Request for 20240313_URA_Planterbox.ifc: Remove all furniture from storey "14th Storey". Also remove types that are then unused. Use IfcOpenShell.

First a look at what the model holds.

```python
import ifcopenshell
import ifcopenshell.util.element

model = ifcopenshell.open("20240313_URA_Planterbox.ifc")
print(model.schema)
storey = next(s for s in model.by_type("IfcBuildingStorey") if s.Name == "14th Storey")
furniture = [e for e in ifcopenshell.util.element.get_decomposition(storey) if e.is_a("IfcFurnishingElement")]
seen = {}
for e in furniture:
    element_type = ifcopenshell.util.element.get_type(e)
    name = element_type.Name if element_type not in (None, e) else None
    seen[name] = seen.get(name, 0) + 1
for name, count in sorted(seen.items(), key=str):
    print(count, "x", name)
```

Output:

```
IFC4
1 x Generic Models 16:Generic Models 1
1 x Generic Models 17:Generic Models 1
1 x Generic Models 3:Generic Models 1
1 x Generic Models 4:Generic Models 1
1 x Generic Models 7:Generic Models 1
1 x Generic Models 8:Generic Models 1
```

```python
import ifcopenshell
import ifcopenshell.api.root
import ifcopenshell.util.element

model = ifcopenshell.open("20240313_URA_Planterbox.ifc")

storey = next(s for s in model.by_type("IfcBuildingStorey") if s.Name == "14th Storey")
furniture = [e for e in ifcopenshell.util.element.get_decomposition(storey) if e.is_a("IfcFurnishingElement")]
types = {ifcopenshell.util.element.get_type(e) for e in furniture} - {None, *furniture}

for e in furniture:
    ifcopenshell.api.root.remove_product(model, product=e)
print(len(furniture), "removed")

unused = [t for t in types if not ifcopenshell.util.element.get_types(t)]
for t in unused:
    ifcopenshell.api.root.remove_product(model, product=t)
print(len(unused), "unused types removed")

model.write("20240313_URA_Planterbox_rev.ifc")
```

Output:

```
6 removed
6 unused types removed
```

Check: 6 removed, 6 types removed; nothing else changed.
